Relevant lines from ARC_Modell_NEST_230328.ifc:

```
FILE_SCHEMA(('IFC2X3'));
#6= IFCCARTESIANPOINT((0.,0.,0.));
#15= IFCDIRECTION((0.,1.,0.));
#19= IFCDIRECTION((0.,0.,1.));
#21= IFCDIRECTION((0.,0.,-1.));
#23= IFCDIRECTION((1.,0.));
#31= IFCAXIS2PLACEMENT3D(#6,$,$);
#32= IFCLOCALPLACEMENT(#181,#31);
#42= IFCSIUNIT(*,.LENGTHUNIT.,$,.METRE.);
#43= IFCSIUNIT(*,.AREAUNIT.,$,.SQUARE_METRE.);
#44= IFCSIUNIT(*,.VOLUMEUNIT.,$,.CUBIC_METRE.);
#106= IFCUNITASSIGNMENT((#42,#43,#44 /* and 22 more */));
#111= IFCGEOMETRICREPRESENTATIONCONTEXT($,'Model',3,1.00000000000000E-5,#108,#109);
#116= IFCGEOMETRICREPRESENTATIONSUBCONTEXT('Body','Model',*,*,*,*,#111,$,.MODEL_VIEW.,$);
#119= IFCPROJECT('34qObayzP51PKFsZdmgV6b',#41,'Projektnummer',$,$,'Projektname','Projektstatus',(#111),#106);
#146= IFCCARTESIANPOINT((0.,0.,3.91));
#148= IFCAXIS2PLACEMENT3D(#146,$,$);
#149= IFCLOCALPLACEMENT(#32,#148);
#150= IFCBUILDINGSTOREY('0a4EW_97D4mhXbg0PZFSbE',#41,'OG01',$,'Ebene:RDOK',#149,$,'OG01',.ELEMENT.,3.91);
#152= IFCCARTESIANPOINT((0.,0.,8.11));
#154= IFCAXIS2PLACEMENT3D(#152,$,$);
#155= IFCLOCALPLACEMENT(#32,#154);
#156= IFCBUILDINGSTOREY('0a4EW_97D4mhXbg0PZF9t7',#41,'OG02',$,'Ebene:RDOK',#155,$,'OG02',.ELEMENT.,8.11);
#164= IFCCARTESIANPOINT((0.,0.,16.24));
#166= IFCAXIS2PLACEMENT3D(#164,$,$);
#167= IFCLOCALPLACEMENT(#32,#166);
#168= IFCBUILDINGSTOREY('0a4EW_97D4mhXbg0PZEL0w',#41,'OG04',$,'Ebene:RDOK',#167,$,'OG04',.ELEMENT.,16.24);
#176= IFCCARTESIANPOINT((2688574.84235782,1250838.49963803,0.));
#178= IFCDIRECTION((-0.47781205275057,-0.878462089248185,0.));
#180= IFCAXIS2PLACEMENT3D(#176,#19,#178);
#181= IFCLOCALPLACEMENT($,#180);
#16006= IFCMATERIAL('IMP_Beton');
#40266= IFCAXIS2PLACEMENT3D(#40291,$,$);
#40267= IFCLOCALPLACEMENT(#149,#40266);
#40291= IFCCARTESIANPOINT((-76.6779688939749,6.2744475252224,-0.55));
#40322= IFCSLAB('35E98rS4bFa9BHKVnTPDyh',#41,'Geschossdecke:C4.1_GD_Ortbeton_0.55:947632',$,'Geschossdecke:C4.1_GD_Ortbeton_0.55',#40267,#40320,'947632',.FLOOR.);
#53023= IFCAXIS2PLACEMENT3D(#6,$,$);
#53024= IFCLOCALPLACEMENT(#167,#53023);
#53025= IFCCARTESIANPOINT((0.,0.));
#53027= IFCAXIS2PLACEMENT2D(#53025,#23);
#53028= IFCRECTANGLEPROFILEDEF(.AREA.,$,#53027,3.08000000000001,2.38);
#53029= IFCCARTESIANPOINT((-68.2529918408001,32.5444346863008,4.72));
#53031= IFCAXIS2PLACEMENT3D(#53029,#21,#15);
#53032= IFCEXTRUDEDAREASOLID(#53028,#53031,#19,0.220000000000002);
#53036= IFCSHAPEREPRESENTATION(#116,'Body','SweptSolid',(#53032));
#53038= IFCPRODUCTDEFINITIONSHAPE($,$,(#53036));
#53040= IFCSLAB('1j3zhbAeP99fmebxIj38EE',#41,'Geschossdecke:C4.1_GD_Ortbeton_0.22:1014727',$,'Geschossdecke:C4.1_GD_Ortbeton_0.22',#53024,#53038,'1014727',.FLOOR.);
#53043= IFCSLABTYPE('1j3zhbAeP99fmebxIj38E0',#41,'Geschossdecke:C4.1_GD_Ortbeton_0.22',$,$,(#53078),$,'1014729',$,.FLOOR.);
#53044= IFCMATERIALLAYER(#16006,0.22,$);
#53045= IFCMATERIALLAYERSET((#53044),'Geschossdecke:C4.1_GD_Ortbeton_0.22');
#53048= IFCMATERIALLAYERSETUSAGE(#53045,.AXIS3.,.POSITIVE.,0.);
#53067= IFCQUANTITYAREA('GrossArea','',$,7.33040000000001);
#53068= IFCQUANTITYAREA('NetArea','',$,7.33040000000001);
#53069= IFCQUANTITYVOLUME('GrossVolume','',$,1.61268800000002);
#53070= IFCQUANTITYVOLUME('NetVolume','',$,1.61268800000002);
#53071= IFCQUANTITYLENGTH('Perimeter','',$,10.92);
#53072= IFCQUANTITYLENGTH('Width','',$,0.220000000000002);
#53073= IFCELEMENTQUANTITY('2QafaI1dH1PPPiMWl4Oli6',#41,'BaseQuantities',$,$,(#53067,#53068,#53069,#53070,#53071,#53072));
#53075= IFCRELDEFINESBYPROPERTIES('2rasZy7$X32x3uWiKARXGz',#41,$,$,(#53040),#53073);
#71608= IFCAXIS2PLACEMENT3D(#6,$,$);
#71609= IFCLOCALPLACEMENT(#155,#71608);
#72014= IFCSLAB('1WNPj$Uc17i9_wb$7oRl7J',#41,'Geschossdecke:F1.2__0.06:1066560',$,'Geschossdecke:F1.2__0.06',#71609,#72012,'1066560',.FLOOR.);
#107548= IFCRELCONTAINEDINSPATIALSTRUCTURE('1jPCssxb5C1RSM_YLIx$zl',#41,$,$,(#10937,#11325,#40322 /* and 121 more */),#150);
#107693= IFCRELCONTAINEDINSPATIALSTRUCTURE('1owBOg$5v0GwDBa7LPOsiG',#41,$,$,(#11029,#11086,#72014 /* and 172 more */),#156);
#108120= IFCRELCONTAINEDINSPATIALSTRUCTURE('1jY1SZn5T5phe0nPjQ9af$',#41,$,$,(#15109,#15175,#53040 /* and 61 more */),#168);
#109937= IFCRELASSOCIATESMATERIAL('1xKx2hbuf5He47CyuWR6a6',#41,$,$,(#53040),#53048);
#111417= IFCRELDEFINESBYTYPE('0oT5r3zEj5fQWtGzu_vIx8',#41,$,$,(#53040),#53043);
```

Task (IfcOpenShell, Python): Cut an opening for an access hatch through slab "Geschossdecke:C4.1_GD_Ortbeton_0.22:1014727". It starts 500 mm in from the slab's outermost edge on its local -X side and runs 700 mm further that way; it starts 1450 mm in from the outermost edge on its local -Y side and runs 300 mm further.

```python
import numpy as np
import ifcopenshell
import ifcopenshell.api.feature
import ifcopenshell.api.geometry
import ifcopenshell.api.pset
import ifcopenshell.api.root
import ifcopenshell.geom
import ifcopenshell.util.element
import ifcopenshell.util.placement
import ifcopenshell.util.representation
import ifcopenshell.util.shape
import ifcopenshell.util.unit

model = ifcopenshell.open("ARC_Modell_NEST_230328.ifc")
unit_scale = ifcopenshell.util.unit.calculate_unit_scale(model)
area_scale = ifcopenshell.util.unit.calculate_unit_scale(model, "AREAUNIT")
volume_scale = ifcopenshell.util.unit.calculate_unit_scale(model, "VOLUMEUNIT")
settings = ifcopenshell.geom.settings()


def volume(element):
    """Net volume in cubic metres, openings subtracted."""
    shape = ifcopenshell.geom.create_shape(settings, element)
    return ifcopenshell.util.shape.get_volume(shape.geometry)


slab = model.by_guid("1j3zhbAeP99fmebxIj38EE")
before = volume(slab)

# Extent in the slab's own axes, in metres. The edges named are its -X and -Y sides.
slab_shape = ifcopenshell.geom.create_shape(settings, slab)
vertices = ifcopenshell.util.shape.get_vertices(slab_shape.geometry)
x_min, y_min, bottom = vertices.min(axis=0)
top = vertices[:, 2].max()

opening = ifcopenshell.api.root.create_entity(model, ifc_class="IfcOpeningElement", name="Access hatch opening")
context = ifcopenshell.util.representation.get_context(model, "Model", "Body", "MODEL_VIEW")
width, depth = 0.7, 0.3
outline = [(0.0, 0.0), (width, 0.0), (width, depth), (0.0, depth), (0.0, 0.0)]
# Overshoot both faces by 50 mm so the cut is clean.
shape = ifcopenshell.api.geometry.add_slab_representation(
    model, context=context, depth=top - bottom + 0.1, polyline=outline
)
ifcopenshell.api.geometry.assign_representation(model, product=opening, representation=shape)

matrix = ifcopenshell.util.placement.get_local_placement(slab.ObjectPlacement)
matrix[:, 3] = matrix @ np.append(np.array([x_min + 0.5, y_min + 1.45, bottom - 0.05]) / unit_scale, 1.0)
ifcopenshell.api.geometry.edit_object_placement(model, product=opening, matrix=matrix, is_si=False)
ifcopenshell.api.feature.add_feature(model, feature=opening, element=slab)

after = volume(slab)

# Update the slab's stored quantities.
qto = model.by_id(ifcopenshell.util.element.get_pset(slab, "BaseQuantities", should_inherit=False)["id"])
ifcopenshell.api.pset.edit_qto(model, qto=qto, properties={
    "NetArea": after / (top - bottom) / area_scale,
    "NetVolume": after / volume_scale,
})

print(f"slab volume {before:.3f} -> {after:.3f} m3")

model.write("ARC_Modell_NEST_230328_v2.ifc")
```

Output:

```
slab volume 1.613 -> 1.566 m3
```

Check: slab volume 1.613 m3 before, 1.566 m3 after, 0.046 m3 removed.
